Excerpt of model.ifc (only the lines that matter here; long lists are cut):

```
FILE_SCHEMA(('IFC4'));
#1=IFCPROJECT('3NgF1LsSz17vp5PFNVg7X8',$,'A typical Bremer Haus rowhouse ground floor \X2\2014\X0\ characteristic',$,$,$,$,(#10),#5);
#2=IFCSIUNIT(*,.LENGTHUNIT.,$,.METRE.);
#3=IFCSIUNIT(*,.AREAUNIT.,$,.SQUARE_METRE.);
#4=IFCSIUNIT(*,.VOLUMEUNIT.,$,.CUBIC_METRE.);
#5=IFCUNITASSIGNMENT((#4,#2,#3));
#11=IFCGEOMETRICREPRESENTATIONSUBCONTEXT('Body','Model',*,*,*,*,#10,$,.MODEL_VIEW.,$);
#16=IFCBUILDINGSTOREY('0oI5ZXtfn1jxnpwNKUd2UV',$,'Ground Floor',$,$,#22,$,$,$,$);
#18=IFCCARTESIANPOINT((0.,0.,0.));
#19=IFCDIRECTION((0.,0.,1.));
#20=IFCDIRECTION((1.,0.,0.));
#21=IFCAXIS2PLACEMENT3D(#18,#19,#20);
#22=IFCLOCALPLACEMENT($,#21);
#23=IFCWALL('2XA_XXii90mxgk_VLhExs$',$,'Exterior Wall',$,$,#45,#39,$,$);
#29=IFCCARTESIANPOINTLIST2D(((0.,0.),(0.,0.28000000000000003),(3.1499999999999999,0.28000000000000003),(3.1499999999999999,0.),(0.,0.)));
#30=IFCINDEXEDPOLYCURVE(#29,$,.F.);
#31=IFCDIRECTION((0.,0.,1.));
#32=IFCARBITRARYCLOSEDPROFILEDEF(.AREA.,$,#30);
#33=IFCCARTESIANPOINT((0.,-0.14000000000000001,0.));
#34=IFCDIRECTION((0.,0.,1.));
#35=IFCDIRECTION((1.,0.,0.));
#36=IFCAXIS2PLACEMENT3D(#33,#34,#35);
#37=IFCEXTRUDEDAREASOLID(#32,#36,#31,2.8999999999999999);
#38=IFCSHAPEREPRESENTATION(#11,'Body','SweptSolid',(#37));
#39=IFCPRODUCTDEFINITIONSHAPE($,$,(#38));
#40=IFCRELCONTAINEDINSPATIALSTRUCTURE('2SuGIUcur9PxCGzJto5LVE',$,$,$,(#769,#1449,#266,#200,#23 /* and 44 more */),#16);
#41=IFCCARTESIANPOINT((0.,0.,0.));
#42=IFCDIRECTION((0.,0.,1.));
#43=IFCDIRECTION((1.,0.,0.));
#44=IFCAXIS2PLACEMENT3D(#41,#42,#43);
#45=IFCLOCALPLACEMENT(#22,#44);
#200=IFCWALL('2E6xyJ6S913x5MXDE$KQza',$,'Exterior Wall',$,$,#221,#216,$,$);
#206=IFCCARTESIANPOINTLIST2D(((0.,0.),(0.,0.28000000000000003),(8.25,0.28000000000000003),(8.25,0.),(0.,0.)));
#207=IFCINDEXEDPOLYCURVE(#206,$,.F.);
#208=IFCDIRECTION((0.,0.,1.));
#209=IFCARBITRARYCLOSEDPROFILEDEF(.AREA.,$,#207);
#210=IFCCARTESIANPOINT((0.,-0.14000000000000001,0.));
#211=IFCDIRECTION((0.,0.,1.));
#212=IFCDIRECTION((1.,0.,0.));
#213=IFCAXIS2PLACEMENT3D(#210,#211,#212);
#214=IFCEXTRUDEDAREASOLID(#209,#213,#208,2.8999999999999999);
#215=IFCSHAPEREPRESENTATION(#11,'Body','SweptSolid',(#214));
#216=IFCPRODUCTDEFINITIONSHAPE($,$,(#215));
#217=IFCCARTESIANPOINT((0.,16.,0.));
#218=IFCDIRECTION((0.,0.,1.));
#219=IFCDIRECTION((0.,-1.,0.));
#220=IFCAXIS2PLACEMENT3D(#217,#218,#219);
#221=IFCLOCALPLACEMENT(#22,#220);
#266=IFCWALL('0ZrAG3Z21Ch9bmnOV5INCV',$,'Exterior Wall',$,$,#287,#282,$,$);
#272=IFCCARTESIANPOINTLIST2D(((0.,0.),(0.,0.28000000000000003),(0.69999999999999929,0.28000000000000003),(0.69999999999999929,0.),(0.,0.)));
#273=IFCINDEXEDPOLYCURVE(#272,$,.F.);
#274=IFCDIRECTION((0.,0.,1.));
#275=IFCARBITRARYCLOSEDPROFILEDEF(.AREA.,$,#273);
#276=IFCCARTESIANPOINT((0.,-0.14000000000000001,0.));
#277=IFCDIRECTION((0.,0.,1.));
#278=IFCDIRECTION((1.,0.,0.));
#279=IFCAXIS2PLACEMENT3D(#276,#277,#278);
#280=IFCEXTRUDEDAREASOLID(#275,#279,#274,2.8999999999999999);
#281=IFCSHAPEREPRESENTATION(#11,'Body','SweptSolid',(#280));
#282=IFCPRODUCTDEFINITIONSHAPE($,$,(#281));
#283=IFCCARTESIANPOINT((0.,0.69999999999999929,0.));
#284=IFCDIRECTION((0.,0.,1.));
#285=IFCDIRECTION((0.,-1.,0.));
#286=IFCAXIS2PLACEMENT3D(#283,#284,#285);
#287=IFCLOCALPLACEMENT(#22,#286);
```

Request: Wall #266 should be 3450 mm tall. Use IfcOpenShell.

```python
import ifcopenshell
import ifcopenshell.geom
import ifcopenshell.util.representation
import ifcopenshell.util.shape

model = ifcopenshell.open("model.ifc")
settings = ifcopenshell.geom.settings()


def volume(element):
    """Net volume in cubic metres, openings subtracted."""
    shape = ifcopenshell.geom.create_shape(settings, element)
    return ifcopenshell.util.shape.get_volume(shape.geometry)


wall = model.by_guid("0ZrAG3Z21Ch9bmnOV5INCV")
before = volume(wall)

body = ifcopenshell.util.representation.get_representation(wall, "Model", "Body")
solid = body.Items[0]
old_height = solid.Depth
solid.Depth = 3.45
after = volume(wall)

print(f"height {old_height:g} -> {solid.Depth:g}, volume {before:.3f} -> {after:.3f} m3")

model.write("model_v2.ifc")
```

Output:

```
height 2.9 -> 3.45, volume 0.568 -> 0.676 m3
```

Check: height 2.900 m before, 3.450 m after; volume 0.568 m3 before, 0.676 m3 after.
